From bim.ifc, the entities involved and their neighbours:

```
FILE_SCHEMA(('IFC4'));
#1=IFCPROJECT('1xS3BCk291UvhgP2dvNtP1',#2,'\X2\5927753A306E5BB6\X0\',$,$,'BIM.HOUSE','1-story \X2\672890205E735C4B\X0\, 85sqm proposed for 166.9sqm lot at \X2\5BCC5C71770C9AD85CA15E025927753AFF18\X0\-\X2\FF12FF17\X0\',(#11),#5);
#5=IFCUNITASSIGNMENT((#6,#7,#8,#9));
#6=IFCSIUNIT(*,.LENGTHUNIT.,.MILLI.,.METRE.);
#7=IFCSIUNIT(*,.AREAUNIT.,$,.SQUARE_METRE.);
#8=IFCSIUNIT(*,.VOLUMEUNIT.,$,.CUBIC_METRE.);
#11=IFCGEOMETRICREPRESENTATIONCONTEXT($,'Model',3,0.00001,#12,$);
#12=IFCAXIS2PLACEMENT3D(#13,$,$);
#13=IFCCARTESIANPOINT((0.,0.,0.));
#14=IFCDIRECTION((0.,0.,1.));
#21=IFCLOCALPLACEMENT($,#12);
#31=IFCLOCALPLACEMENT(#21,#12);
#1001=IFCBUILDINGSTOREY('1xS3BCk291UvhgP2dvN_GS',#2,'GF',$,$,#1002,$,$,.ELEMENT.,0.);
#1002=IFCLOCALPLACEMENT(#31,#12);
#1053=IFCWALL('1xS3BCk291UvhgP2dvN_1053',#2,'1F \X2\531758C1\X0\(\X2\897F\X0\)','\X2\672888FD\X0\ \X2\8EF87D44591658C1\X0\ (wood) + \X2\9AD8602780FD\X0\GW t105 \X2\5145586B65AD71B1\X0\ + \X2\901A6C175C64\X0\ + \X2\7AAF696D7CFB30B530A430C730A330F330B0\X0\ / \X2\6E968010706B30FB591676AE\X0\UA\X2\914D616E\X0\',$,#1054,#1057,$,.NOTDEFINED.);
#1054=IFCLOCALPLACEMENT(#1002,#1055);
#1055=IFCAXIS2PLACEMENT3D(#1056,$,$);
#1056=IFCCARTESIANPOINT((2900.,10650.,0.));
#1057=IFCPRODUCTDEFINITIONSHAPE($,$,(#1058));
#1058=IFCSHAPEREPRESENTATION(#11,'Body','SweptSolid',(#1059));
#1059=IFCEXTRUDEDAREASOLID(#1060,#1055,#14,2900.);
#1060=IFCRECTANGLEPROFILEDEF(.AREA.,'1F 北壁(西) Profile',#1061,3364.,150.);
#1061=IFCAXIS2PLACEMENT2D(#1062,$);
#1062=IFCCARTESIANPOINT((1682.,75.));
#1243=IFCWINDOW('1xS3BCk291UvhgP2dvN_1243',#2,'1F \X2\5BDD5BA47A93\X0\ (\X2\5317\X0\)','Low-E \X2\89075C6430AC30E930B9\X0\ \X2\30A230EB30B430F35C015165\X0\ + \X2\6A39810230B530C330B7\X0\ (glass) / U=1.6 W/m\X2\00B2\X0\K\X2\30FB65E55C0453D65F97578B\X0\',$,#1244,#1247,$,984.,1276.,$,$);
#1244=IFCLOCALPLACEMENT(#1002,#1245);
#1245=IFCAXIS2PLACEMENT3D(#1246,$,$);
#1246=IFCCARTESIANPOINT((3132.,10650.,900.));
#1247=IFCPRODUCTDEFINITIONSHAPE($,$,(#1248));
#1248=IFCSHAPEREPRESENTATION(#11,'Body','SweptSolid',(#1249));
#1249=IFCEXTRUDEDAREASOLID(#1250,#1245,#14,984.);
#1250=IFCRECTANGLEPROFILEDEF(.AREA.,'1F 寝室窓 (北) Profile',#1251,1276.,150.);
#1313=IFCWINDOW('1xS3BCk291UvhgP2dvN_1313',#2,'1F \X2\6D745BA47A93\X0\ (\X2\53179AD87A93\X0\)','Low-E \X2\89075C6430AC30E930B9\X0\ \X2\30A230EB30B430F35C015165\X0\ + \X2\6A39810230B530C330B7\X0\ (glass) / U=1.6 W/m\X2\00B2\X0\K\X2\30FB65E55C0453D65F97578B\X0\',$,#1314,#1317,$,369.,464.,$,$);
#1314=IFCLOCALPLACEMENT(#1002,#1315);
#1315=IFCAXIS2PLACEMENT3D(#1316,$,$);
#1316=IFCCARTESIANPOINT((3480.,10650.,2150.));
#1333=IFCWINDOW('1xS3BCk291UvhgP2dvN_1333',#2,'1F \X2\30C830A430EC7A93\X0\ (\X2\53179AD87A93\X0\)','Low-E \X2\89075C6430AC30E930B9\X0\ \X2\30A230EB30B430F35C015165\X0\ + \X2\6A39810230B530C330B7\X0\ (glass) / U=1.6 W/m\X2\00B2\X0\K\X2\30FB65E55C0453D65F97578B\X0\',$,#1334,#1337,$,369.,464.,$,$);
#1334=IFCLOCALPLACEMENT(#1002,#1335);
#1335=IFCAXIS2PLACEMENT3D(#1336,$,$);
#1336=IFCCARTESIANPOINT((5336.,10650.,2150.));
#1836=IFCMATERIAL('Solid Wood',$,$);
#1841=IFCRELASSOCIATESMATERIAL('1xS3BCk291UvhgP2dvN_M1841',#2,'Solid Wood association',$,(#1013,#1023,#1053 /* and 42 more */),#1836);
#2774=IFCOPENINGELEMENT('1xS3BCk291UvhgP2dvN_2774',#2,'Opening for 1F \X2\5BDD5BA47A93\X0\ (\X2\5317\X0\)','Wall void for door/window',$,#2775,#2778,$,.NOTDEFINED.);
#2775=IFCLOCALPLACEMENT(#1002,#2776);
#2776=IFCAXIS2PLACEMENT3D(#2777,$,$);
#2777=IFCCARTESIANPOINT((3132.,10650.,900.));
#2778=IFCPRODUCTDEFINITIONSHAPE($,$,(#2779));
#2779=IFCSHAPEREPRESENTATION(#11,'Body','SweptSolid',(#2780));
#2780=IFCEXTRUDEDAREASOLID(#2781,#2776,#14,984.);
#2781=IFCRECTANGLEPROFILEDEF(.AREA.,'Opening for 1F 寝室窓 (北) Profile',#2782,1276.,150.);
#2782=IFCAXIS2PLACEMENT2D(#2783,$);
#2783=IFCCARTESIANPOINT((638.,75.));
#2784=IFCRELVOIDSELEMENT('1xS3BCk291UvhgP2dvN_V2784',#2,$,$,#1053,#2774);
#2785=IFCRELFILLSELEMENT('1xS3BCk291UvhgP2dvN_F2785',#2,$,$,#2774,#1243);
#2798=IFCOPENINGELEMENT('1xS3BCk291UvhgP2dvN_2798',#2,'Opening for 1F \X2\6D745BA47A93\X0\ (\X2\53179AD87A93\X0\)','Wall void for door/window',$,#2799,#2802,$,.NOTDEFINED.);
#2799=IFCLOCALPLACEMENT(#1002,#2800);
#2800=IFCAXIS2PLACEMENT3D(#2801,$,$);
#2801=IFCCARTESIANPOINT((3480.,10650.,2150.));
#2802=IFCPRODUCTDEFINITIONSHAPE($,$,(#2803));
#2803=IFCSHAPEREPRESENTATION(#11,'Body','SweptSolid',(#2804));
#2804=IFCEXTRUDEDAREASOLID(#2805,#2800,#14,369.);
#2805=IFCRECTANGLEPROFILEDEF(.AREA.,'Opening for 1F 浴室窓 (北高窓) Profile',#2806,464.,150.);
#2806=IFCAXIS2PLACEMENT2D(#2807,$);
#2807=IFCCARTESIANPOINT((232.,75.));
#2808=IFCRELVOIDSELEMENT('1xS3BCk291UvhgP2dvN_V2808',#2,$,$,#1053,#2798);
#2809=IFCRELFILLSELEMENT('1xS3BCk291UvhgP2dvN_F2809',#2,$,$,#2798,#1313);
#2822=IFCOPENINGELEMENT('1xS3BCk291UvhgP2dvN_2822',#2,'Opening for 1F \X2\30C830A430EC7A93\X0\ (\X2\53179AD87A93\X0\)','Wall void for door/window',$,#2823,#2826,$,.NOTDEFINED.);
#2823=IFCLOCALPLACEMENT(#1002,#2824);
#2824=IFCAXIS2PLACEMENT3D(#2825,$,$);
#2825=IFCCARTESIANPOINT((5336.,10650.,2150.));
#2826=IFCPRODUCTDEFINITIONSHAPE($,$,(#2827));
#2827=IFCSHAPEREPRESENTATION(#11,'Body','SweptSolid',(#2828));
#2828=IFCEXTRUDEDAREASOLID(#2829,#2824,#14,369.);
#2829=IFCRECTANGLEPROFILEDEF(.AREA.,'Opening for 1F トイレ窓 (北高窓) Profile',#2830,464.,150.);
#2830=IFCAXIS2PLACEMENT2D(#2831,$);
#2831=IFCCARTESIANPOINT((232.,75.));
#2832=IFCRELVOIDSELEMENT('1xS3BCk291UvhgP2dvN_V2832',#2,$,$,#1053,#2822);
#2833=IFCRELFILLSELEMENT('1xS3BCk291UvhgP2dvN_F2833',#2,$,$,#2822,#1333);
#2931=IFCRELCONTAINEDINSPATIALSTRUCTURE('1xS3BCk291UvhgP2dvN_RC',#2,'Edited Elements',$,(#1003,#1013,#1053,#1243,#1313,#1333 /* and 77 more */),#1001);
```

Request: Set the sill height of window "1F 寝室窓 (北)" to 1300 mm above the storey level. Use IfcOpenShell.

```python
import numpy as np
import ifcopenshell
import ifcopenshell.api.geometry
import ifcopenshell.geom
import ifcopenshell.util.element
import ifcopenshell.util.placement
import ifcopenshell.util.shape
import ifcopenshell.util.unit

model = ifcopenshell.open("bim.ifc")
unit_scale = ifcopenshell.util.unit.calculate_unit_scale(model)

window = model.by_guid("1xS3BCk291UvhgP2dvN_1243")
opening = window.FillsVoids[0].RelatingOpeningElement
storey = ifcopenshell.util.element.get_container(window, ifc_class="IfcBuildingStorey")
level = ifcopenshell.util.placement.get_local_placement(storey.ObjectPlacement)[2, 3]

# The opening's origin need not be at the sill, so measure its lowest point.
shape = ifcopenshell.geom.create_shape(ifcopenshell.geom.settings(), opening)
bottom = ifcopenshell.util.shape.get_shape_bottom_elevation(shape, shape.geometry) / unit_scale
dz = level + 1300.0 - bottom

shift = np.array([0.0, 0.0, dz])
# The window is not placed relative to its opening, so move both.
for product in (opening, window):
    matrix = ifcopenshell.util.placement.get_local_placement(product.ObjectPlacement)
    matrix[:3, 3] += shift
    ifcopenshell.api.geometry.edit_object_placement(model, product=product, matrix=matrix, is_si=False)

print(f"moved by {dz * unit_scale:+.3f} m")

model.write("bim_edited.ifc")
```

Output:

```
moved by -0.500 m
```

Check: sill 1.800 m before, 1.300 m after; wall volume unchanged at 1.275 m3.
